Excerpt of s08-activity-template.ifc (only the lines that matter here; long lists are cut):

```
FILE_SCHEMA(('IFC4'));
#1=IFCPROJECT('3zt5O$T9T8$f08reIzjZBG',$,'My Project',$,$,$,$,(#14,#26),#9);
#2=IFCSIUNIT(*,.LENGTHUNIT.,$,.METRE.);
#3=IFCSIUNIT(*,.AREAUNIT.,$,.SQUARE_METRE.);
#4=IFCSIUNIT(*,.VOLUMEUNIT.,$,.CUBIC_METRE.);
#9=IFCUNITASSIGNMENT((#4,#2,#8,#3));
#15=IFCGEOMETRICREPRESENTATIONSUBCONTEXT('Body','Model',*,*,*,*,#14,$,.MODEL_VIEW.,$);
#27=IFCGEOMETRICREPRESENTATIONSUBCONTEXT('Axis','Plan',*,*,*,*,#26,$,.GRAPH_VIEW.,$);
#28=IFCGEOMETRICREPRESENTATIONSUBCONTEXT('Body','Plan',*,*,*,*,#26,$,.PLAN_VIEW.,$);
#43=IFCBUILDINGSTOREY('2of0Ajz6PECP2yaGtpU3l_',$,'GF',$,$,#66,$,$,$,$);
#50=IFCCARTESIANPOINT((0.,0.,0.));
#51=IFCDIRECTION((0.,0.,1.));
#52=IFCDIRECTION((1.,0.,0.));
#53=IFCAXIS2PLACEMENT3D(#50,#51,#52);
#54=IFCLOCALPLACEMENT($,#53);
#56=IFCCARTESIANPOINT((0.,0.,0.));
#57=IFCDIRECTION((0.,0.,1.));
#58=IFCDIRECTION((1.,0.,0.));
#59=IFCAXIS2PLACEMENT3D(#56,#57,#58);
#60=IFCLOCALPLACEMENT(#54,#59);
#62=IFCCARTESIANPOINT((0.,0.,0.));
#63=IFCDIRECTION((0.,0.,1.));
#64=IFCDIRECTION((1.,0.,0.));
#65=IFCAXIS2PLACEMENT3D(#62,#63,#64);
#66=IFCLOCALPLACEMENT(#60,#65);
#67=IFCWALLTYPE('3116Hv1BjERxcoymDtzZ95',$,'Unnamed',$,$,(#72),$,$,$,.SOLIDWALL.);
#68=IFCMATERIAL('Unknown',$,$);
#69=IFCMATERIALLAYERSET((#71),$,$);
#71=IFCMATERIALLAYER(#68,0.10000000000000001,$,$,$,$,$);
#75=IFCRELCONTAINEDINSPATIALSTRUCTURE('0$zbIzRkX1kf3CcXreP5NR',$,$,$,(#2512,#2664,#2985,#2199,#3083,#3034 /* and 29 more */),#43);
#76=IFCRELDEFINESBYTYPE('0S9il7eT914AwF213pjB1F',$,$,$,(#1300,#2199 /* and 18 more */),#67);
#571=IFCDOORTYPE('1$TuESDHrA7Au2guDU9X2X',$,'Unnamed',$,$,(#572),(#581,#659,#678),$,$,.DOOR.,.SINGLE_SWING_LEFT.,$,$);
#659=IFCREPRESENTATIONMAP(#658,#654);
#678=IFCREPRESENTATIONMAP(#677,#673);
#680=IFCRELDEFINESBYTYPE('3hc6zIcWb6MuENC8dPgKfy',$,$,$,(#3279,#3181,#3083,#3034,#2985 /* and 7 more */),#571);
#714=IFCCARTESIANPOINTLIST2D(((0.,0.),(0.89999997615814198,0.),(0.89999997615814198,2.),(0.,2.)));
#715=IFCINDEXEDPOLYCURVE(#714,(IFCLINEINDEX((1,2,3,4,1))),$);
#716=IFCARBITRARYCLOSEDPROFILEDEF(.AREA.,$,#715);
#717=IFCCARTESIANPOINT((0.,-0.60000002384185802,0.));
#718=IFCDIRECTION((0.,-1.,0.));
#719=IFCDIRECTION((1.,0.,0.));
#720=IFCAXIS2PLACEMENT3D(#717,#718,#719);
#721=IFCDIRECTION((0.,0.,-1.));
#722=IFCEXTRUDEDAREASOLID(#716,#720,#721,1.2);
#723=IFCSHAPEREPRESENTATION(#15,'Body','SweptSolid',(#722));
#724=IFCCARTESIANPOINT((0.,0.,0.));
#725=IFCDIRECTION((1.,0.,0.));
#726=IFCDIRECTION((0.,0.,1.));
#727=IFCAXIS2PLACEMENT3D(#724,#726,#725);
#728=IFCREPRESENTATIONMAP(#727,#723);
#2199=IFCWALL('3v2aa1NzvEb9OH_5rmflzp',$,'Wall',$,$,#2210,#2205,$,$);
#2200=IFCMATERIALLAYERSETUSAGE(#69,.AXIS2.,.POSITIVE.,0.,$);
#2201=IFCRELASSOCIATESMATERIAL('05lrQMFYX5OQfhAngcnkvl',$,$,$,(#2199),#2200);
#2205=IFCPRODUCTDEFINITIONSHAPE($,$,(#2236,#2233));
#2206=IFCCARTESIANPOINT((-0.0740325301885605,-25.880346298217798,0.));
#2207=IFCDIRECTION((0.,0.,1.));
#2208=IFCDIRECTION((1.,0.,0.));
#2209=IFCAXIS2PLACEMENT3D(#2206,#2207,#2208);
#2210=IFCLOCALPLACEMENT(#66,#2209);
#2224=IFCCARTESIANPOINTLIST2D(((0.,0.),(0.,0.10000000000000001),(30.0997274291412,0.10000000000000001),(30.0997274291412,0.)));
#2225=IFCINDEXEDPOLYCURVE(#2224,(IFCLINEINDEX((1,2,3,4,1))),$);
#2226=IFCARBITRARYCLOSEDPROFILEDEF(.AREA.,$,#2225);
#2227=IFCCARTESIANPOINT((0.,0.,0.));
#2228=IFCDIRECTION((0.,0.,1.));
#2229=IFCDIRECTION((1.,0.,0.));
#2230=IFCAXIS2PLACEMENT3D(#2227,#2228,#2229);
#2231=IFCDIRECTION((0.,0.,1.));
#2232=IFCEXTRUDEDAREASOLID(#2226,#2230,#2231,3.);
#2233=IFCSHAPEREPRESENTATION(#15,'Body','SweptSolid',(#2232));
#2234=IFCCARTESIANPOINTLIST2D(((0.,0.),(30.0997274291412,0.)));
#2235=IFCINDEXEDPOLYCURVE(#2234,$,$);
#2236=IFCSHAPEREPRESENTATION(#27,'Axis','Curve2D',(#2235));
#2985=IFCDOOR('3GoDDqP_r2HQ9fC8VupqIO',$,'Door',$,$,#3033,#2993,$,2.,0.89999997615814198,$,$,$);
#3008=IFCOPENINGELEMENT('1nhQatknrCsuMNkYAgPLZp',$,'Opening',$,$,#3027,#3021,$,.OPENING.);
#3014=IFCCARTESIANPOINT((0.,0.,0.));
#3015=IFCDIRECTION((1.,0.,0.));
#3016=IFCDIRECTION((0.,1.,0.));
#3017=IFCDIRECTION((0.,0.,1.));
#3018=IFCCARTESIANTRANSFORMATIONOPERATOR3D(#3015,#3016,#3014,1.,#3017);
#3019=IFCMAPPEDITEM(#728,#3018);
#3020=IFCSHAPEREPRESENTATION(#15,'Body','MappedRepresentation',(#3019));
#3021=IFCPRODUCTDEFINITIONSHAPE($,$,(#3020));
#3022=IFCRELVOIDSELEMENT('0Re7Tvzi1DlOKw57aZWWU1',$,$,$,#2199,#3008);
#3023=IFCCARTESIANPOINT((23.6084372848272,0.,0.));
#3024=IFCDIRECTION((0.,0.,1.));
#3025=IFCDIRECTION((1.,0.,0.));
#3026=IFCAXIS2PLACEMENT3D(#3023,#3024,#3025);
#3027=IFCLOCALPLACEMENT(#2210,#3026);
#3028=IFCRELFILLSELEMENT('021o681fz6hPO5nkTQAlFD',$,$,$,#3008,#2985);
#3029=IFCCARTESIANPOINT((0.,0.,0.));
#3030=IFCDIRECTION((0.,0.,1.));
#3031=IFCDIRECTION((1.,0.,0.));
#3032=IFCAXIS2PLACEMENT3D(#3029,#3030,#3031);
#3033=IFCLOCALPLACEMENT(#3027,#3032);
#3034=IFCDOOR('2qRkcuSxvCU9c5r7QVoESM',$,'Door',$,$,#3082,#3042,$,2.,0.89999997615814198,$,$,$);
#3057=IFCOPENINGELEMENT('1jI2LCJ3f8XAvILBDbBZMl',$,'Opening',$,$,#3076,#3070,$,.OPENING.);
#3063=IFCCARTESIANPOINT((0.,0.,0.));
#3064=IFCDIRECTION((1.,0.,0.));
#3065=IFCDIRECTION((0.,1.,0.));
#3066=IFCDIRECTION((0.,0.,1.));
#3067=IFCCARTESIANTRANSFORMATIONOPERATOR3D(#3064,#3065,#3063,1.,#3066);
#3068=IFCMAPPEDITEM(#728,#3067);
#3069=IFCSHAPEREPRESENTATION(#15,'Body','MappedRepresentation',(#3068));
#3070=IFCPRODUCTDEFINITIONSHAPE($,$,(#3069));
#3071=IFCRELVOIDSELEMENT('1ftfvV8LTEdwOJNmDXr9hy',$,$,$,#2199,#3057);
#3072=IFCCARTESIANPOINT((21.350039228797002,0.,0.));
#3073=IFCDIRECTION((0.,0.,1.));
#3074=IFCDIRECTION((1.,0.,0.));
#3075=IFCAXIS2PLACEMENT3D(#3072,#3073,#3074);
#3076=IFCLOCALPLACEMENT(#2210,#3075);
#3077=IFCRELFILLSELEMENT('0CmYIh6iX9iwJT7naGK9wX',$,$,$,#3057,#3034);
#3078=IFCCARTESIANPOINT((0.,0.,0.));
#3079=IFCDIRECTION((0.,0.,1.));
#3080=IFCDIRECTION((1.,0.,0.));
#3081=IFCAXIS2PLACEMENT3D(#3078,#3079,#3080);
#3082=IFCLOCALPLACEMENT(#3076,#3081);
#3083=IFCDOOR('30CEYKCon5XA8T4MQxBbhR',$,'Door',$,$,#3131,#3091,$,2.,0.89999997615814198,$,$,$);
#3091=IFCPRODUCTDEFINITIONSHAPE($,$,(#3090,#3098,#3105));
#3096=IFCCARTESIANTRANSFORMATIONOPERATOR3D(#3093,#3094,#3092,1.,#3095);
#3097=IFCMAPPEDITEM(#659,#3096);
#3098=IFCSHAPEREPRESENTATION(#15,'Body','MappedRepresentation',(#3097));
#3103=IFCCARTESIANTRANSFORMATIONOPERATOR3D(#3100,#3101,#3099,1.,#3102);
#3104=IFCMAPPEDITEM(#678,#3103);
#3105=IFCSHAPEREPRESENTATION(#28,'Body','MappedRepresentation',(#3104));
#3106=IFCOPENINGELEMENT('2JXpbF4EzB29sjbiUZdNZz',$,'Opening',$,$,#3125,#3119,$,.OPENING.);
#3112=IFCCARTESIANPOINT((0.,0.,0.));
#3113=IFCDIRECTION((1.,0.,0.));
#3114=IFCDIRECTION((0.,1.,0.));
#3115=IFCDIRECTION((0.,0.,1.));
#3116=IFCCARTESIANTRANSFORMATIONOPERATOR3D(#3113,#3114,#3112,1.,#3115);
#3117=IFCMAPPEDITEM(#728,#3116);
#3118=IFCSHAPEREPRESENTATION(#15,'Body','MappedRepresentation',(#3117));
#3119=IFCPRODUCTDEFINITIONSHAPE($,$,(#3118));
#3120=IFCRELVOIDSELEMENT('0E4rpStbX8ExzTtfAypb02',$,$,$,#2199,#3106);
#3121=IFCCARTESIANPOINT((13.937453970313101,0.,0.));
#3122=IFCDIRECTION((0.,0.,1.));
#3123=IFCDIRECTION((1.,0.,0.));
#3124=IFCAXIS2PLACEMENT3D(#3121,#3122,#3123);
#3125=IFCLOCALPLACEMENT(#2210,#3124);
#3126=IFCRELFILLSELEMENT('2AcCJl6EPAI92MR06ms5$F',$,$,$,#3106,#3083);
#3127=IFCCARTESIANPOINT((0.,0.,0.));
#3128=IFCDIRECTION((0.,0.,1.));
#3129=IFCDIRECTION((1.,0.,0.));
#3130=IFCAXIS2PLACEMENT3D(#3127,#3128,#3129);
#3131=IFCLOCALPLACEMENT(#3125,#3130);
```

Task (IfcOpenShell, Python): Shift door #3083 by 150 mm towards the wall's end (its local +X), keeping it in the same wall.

```python
import ifcopenshell
import ifcopenshell.api.geometry
import ifcopenshell.util.placement
import ifcopenshell.util.unit

model = ifcopenshell.open("s08-activity-template.ifc")
unit_scale = ifcopenshell.util.unit.calculate_unit_scale(model)

door = model.by_guid("30CEYKCon5XA8T4MQxBbhR")
opening = door.FillsVoids[0].RelatingOpeningElement
wall = opening.VoidsElements[0].RelatingBuildingElement

wall_matrix = ifcopenshell.util.placement.get_local_placement(wall.ObjectPlacement)
shift = wall_matrix[:3, 0] * 0.15 / unit_scale
before = ifcopenshell.util.placement.get_local_placement(door.ObjectPlacement)[:3, 3].copy()

# The door is placed relative to its opening, so it follows when the opening moves.
matrix = ifcopenshell.util.placement.get_local_placement(opening.ObjectPlacement)
matrix[:3, 3] += shift
ifcopenshell.api.geometry.edit_object_placement(
    model, product=opening, matrix=matrix, is_si=False, should_transform_children=True
)

after = ifcopenshell.util.placement.get_local_placement(door.ObjectPlacement)[:3, 3]
print("door moved by", (after - before).round(3) + 0.0)

model.write("s08-activity-template_edited.ifc")
```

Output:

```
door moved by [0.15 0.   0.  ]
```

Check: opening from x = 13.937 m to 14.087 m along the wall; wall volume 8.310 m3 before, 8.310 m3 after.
